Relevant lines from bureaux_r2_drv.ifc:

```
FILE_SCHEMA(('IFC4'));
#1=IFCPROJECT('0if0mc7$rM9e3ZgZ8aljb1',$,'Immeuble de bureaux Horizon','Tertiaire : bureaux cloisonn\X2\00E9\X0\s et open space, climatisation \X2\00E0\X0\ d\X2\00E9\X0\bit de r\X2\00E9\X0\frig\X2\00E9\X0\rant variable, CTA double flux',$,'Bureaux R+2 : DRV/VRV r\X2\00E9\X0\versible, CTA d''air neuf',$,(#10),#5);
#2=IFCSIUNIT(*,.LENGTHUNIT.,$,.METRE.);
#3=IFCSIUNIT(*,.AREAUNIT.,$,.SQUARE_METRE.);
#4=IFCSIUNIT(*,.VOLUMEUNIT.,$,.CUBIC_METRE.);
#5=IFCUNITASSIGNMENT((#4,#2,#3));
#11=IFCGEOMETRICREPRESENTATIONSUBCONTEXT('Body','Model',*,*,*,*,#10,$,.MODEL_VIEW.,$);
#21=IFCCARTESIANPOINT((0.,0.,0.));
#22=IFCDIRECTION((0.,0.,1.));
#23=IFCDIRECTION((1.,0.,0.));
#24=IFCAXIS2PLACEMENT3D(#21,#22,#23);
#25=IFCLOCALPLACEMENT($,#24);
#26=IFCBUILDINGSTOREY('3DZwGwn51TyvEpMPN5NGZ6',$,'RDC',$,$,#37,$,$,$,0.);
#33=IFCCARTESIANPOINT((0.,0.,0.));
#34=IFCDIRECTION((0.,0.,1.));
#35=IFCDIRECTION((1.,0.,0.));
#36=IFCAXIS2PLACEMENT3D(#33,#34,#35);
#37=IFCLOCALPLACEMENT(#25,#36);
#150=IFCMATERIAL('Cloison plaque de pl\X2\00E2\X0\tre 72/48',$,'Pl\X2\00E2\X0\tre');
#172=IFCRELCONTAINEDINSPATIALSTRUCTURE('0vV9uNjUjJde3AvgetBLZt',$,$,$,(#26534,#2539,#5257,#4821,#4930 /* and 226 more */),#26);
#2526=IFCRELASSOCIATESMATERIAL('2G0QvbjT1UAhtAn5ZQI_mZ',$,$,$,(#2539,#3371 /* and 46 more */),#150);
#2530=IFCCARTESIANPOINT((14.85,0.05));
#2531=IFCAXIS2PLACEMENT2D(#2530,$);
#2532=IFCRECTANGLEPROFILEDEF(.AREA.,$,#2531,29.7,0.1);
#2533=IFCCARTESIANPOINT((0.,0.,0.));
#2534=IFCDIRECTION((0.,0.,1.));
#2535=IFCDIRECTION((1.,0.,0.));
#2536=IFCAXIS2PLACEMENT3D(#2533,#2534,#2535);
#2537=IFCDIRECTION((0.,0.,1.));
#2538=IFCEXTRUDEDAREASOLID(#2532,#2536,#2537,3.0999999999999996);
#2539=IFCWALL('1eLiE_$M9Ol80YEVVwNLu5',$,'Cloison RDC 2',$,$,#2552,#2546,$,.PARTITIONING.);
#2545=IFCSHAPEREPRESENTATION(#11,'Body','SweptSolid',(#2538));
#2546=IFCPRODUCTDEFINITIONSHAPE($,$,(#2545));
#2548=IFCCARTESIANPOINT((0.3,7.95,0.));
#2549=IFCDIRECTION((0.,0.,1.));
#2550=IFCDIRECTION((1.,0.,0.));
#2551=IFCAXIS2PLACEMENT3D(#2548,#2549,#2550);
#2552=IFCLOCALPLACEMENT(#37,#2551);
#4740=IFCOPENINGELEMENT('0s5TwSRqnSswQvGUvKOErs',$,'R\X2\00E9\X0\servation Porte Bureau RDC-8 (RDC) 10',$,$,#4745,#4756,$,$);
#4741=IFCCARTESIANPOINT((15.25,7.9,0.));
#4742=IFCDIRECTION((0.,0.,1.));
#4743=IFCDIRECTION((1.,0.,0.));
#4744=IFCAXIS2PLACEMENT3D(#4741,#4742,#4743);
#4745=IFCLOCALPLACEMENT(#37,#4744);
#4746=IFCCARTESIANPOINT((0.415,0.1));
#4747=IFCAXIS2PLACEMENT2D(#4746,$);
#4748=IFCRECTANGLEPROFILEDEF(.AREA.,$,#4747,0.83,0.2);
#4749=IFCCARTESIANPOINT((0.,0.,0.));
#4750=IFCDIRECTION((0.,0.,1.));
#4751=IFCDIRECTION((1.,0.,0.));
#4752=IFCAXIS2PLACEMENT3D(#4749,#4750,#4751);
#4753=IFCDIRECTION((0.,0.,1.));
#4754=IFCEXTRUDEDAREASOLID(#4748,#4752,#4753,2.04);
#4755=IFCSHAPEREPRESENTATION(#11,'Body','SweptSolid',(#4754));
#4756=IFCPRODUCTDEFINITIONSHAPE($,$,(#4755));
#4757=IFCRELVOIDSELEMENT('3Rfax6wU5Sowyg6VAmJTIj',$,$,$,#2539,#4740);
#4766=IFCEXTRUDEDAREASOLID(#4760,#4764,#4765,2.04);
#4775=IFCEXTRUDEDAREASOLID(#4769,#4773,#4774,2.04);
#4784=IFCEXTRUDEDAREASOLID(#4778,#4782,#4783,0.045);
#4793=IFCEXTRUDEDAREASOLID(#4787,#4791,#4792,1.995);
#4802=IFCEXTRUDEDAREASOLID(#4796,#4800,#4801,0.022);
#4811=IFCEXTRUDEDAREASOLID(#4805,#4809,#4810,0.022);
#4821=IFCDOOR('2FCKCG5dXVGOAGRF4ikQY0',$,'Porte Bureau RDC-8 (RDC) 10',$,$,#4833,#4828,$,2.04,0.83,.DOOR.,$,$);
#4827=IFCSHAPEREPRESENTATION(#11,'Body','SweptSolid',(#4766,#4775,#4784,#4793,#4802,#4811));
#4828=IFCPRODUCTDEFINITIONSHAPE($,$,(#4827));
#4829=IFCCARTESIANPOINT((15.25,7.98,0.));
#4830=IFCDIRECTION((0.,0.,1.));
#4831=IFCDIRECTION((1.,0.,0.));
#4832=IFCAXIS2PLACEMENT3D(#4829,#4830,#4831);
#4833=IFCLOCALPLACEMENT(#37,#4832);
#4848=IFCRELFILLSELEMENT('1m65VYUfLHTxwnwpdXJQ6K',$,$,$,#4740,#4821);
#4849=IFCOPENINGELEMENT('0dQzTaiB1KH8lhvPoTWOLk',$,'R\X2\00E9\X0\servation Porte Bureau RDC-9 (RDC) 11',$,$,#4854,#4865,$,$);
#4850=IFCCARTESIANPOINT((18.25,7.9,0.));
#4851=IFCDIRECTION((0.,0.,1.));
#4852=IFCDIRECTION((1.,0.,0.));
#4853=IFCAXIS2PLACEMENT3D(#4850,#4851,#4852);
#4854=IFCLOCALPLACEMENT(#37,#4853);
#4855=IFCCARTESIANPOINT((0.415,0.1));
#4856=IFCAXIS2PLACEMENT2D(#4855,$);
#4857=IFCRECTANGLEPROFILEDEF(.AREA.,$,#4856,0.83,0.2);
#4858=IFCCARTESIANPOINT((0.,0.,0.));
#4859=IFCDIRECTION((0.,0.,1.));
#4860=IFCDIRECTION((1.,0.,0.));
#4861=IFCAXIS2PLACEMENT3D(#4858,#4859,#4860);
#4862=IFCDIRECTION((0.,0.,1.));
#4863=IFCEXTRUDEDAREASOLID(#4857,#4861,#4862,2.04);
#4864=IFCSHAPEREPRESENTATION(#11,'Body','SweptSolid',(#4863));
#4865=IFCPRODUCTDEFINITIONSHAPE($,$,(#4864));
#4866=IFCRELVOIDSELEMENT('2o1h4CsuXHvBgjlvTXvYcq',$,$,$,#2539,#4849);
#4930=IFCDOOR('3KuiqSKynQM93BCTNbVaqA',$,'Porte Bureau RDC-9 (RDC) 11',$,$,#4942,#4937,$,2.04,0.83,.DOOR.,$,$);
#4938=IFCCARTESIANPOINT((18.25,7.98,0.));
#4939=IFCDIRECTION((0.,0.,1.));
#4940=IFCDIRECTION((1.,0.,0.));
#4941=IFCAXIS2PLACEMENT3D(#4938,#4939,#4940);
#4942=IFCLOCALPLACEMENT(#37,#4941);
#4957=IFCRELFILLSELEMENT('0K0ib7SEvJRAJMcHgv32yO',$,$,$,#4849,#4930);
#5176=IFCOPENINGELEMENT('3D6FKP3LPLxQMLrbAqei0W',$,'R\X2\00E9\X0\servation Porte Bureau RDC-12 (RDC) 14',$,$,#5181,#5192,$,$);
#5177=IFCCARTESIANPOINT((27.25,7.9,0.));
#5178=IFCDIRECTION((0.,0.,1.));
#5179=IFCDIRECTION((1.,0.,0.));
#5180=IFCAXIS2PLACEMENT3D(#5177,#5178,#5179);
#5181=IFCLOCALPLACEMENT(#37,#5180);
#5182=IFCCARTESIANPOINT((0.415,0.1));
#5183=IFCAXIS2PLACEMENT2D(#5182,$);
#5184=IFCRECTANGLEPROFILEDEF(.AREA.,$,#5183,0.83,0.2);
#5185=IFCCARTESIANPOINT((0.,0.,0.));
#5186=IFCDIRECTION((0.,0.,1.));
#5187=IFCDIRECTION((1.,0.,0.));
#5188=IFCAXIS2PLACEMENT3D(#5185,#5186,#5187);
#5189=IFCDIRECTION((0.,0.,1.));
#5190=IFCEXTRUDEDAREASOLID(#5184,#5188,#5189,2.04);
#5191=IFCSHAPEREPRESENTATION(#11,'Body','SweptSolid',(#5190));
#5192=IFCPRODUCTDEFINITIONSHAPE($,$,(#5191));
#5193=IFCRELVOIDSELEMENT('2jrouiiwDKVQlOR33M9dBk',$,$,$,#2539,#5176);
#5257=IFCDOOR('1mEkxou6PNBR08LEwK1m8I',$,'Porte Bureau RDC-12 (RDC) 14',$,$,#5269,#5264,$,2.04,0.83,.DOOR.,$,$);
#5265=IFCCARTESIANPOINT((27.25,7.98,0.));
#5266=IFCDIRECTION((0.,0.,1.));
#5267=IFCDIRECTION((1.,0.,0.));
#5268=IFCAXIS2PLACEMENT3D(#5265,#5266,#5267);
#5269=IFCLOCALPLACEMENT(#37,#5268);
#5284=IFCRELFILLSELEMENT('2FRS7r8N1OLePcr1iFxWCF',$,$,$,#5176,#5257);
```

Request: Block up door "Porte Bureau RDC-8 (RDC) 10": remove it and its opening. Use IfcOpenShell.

```python
import ifcopenshell
import ifcopenshell.api.feature
import ifcopenshell.api.root
import ifcopenshell.geom
import ifcopenshell.util.shape

model = ifcopenshell.open("bureaux_r2_drv.ifc")
settings = ifcopenshell.geom.settings()


def volume(element):
    """Net volume in cubic metres, openings subtracted."""
    shape = ifcopenshell.geom.create_shape(settings, element)
    return ifcopenshell.util.shape.get_volume(shape.geometry)


door = model.by_guid("2FCKCG5dXVGOAGRF4ikQY0")
opening = door.FillsVoids[0].RelatingOpeningElement
wall = opening.VoidsElements[0].RelatingBuildingElement
before = volume(wall)

ifcopenshell.api.root.remove_product(model, product=door)
ifcopenshell.api.feature.remove_feature(model, feature=opening)

after = volume(wall)

print(f"wall volume {before:.3f} -> {after:.3f} m3")

model.write("bureaux_r2_drv_edited.ifc")
```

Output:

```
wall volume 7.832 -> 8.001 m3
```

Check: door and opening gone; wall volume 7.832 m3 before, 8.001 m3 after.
